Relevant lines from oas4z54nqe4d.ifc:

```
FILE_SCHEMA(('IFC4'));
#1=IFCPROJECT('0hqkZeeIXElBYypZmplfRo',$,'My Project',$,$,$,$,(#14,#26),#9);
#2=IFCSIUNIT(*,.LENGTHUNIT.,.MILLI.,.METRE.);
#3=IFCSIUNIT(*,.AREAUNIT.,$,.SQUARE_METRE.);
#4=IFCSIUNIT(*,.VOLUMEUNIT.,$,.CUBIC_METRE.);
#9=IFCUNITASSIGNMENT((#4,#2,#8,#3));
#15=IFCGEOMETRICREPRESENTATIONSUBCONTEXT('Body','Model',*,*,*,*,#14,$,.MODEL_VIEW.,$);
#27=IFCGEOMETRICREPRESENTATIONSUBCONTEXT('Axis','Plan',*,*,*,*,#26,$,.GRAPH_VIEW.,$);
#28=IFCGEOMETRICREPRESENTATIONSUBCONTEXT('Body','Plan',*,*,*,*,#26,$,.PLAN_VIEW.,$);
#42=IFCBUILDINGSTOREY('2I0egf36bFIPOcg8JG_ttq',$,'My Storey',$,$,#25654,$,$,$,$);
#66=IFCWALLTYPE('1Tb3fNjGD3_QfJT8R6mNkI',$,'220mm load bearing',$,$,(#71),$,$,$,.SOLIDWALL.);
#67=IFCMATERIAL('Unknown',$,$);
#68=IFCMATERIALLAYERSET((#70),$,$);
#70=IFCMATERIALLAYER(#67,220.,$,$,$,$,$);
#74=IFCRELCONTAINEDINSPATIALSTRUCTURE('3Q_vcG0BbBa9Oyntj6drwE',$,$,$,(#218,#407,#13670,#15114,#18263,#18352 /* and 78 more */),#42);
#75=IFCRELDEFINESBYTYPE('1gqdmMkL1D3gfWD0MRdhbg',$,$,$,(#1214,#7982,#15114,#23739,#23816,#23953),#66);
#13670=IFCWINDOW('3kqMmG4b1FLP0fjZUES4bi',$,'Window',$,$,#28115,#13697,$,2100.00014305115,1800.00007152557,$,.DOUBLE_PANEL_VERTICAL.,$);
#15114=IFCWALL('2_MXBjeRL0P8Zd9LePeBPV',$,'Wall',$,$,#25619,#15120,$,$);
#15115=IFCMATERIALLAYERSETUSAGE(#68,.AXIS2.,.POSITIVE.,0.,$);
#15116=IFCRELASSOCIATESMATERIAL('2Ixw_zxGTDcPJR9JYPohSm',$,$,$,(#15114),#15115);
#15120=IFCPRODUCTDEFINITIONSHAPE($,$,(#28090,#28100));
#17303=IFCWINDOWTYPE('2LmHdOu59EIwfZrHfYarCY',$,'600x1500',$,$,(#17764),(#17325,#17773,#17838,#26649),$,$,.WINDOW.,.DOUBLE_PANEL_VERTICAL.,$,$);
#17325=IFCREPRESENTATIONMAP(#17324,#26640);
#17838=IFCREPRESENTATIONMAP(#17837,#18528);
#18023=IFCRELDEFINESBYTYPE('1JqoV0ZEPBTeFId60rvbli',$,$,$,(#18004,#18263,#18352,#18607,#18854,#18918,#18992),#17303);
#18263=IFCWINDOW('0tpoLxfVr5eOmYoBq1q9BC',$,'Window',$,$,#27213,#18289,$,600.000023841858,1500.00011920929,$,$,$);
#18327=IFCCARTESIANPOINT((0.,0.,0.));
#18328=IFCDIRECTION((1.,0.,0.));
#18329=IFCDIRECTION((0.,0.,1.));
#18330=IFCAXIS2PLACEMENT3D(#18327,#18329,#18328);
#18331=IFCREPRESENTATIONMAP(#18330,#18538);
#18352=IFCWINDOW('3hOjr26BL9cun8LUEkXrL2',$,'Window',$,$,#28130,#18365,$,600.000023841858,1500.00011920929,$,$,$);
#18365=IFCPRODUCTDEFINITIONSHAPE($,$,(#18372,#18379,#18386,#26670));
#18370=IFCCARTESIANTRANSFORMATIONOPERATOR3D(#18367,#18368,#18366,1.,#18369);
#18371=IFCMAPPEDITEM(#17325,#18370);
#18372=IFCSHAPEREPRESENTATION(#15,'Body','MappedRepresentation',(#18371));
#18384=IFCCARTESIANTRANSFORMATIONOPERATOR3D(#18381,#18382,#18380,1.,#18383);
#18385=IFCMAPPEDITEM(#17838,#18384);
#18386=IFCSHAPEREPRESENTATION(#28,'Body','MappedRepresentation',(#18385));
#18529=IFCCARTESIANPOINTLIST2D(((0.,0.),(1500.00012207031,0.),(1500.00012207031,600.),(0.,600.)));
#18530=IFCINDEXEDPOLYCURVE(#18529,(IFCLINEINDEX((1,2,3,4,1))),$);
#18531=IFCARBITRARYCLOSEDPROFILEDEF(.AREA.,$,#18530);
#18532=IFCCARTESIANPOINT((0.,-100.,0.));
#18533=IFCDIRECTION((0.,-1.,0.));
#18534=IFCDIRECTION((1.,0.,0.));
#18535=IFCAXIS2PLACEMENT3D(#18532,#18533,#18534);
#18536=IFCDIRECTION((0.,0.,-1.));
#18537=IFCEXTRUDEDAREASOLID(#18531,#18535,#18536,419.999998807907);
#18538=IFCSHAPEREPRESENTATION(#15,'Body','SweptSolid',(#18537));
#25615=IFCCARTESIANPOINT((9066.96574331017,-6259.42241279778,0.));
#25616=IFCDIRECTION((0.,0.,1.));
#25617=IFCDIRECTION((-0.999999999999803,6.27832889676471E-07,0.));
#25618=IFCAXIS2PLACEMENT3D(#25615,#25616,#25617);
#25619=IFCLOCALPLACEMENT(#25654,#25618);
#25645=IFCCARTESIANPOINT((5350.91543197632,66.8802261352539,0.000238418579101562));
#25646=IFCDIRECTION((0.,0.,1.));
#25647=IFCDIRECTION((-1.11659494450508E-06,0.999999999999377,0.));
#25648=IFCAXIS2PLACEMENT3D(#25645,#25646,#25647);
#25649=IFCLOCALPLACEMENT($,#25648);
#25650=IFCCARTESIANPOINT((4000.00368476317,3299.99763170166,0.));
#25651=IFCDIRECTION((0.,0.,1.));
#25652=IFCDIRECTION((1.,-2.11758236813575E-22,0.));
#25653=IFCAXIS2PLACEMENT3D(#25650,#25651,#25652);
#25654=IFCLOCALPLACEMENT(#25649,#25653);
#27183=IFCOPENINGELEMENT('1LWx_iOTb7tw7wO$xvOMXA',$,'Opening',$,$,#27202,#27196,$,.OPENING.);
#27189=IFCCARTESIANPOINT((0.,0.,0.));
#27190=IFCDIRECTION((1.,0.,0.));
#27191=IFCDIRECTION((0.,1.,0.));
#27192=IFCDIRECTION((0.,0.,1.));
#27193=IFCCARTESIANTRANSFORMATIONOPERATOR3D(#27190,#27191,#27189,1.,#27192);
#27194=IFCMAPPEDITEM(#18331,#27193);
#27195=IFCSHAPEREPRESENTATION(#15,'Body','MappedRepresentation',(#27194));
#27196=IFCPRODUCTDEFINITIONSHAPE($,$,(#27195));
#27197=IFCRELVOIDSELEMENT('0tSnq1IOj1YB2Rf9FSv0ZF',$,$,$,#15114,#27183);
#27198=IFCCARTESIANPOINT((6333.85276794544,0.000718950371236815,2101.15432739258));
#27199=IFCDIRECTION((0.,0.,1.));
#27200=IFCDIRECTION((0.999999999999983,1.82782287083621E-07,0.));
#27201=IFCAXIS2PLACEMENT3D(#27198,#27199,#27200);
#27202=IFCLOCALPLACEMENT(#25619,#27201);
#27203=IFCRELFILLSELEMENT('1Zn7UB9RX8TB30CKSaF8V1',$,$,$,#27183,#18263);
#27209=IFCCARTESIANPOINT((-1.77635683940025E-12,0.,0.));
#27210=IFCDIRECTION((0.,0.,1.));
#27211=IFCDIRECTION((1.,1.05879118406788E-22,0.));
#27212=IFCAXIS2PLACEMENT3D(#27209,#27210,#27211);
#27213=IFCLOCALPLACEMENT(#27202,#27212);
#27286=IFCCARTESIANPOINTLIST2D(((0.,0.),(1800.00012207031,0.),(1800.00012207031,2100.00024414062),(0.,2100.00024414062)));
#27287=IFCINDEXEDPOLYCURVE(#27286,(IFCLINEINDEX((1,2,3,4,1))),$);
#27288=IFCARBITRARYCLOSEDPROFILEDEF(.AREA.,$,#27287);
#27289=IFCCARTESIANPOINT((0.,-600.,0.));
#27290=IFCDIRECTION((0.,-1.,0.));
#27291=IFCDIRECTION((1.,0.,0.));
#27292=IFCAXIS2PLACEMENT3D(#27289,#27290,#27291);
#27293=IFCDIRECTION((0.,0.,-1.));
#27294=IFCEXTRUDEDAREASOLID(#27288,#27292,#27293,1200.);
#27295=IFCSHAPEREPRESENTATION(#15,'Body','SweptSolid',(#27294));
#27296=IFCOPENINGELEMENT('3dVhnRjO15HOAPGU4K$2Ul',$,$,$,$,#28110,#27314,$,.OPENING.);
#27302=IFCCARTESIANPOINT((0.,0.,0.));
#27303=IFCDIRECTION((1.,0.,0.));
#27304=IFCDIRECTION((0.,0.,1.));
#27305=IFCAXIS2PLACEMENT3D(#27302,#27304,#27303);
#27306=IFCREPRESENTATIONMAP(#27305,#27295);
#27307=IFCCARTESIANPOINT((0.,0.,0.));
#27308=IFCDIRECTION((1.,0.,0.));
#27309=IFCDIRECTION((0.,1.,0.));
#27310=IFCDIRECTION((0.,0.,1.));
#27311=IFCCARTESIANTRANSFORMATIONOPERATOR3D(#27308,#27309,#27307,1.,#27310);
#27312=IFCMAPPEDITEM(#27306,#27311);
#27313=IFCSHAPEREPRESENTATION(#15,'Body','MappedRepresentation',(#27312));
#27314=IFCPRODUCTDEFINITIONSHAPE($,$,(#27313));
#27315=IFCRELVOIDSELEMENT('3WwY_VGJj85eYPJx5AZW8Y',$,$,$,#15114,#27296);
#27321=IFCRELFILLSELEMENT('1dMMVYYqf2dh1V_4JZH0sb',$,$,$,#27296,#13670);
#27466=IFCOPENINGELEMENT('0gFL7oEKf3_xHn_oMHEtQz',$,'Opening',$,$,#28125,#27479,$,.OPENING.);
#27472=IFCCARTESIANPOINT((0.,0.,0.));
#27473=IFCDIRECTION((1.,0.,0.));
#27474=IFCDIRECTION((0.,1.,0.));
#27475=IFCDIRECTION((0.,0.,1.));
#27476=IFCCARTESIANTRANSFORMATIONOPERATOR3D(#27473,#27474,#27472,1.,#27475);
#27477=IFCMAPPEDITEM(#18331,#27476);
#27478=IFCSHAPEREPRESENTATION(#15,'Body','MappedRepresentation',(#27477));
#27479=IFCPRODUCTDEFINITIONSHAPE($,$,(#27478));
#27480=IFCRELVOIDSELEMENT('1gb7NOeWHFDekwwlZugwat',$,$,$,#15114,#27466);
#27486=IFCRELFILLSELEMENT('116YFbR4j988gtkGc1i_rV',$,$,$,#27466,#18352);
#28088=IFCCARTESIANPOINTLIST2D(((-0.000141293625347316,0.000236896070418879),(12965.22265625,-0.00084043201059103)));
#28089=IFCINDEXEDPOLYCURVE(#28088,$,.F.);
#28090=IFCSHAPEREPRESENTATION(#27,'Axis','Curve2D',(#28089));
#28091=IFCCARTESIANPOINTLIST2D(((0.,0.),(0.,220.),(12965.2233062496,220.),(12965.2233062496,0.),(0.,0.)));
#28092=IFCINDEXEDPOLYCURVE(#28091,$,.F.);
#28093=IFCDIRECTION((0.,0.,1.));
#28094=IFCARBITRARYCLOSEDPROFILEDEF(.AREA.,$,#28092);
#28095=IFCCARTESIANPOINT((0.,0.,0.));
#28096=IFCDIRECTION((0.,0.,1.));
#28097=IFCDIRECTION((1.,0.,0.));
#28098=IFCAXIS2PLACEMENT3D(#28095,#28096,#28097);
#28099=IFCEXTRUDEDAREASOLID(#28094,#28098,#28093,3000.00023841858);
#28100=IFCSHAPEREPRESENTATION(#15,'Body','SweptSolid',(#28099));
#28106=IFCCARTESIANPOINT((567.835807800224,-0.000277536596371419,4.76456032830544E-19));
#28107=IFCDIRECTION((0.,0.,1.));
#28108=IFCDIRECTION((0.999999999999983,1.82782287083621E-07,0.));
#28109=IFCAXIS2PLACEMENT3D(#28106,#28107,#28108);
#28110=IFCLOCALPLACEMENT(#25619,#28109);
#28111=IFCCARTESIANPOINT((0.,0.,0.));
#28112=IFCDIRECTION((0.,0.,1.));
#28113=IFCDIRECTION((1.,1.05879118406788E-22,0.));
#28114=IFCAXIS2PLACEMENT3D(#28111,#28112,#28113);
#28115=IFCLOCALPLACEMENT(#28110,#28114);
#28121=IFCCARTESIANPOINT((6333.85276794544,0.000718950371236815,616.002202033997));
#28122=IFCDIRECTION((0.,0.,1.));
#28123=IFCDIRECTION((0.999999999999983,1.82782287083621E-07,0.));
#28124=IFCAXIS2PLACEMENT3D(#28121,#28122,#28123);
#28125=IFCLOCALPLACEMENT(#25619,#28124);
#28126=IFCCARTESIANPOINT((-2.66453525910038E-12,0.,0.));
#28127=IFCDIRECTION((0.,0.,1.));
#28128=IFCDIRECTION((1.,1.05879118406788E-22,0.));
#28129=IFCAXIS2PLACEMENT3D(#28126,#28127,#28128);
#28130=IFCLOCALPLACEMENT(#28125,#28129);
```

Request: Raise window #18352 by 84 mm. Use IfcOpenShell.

```python
import numpy as np
import ifcopenshell
import ifcopenshell.api.geometry
import ifcopenshell.util.placement
import ifcopenshell.util.unit

model = ifcopenshell.open("oas4z54nqe4d.ifc")
unit_scale = ifcopenshell.util.unit.calculate_unit_scale(model)

window = model.by_guid("3hOjr26BL9cun8LUEkXrL2")
opening = window.FillsVoids[0].RelatingOpeningElement
dz = 84.0

shift = np.array([0.0, 0.0, dz])
# The window is placed relative to its opening, so it follows when the opening moves.
matrix = ifcopenshell.util.placement.get_local_placement(opening.ObjectPlacement)
matrix[:3, 3] += shift
ifcopenshell.api.geometry.edit_object_placement(
    model, product=opening, matrix=matrix, is_si=False, should_transform_children=True
)

print(f"moved by {dz * unit_scale:+.3f} m")

model.write("oas4z54nqe4d_v2.ifc")
```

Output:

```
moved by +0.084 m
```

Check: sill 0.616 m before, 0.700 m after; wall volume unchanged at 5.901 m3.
